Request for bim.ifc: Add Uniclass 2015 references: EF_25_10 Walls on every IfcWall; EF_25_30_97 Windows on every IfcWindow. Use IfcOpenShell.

First a look at what the model holds.

```python
import ifcopenshell

model = ifcopenshell.open("bim.ifc")
print(model.schema)
print("classifications:", [c.Name for c in model.by_type("IfcClassification")])
for ifc_class in ("IfcDoor", "IfcRoof", "IfcStair", "IfcWall", "IfcWindow"):
    print(ifc_class, len(model.by_type(ifc_class)))
```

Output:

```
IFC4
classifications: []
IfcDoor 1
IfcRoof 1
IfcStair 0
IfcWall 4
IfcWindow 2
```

```python
import ifcopenshell
import ifcopenshell.api.classification

model = ifcopenshell.open("bim.ifc")

system = ifcopenshell.api.classification.add_classification(model, classification="Uniclass 2015")

codes = {
    "IfcWall": ("EF_25_10", "Walls"),
    "IfcWindow": ("EF_25_30_97", "Windows"),
}
for ifc_class, (code, name) in codes.items():
    products = model.by_type(ifc_class)
    ifcopenshell.api.classification.add_reference(
        model, products=products, classification=system, identification=code, name=name
    )
    print(code, len(products))

model.write("bim-out.ifc")
```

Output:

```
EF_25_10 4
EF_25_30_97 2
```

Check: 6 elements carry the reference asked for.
